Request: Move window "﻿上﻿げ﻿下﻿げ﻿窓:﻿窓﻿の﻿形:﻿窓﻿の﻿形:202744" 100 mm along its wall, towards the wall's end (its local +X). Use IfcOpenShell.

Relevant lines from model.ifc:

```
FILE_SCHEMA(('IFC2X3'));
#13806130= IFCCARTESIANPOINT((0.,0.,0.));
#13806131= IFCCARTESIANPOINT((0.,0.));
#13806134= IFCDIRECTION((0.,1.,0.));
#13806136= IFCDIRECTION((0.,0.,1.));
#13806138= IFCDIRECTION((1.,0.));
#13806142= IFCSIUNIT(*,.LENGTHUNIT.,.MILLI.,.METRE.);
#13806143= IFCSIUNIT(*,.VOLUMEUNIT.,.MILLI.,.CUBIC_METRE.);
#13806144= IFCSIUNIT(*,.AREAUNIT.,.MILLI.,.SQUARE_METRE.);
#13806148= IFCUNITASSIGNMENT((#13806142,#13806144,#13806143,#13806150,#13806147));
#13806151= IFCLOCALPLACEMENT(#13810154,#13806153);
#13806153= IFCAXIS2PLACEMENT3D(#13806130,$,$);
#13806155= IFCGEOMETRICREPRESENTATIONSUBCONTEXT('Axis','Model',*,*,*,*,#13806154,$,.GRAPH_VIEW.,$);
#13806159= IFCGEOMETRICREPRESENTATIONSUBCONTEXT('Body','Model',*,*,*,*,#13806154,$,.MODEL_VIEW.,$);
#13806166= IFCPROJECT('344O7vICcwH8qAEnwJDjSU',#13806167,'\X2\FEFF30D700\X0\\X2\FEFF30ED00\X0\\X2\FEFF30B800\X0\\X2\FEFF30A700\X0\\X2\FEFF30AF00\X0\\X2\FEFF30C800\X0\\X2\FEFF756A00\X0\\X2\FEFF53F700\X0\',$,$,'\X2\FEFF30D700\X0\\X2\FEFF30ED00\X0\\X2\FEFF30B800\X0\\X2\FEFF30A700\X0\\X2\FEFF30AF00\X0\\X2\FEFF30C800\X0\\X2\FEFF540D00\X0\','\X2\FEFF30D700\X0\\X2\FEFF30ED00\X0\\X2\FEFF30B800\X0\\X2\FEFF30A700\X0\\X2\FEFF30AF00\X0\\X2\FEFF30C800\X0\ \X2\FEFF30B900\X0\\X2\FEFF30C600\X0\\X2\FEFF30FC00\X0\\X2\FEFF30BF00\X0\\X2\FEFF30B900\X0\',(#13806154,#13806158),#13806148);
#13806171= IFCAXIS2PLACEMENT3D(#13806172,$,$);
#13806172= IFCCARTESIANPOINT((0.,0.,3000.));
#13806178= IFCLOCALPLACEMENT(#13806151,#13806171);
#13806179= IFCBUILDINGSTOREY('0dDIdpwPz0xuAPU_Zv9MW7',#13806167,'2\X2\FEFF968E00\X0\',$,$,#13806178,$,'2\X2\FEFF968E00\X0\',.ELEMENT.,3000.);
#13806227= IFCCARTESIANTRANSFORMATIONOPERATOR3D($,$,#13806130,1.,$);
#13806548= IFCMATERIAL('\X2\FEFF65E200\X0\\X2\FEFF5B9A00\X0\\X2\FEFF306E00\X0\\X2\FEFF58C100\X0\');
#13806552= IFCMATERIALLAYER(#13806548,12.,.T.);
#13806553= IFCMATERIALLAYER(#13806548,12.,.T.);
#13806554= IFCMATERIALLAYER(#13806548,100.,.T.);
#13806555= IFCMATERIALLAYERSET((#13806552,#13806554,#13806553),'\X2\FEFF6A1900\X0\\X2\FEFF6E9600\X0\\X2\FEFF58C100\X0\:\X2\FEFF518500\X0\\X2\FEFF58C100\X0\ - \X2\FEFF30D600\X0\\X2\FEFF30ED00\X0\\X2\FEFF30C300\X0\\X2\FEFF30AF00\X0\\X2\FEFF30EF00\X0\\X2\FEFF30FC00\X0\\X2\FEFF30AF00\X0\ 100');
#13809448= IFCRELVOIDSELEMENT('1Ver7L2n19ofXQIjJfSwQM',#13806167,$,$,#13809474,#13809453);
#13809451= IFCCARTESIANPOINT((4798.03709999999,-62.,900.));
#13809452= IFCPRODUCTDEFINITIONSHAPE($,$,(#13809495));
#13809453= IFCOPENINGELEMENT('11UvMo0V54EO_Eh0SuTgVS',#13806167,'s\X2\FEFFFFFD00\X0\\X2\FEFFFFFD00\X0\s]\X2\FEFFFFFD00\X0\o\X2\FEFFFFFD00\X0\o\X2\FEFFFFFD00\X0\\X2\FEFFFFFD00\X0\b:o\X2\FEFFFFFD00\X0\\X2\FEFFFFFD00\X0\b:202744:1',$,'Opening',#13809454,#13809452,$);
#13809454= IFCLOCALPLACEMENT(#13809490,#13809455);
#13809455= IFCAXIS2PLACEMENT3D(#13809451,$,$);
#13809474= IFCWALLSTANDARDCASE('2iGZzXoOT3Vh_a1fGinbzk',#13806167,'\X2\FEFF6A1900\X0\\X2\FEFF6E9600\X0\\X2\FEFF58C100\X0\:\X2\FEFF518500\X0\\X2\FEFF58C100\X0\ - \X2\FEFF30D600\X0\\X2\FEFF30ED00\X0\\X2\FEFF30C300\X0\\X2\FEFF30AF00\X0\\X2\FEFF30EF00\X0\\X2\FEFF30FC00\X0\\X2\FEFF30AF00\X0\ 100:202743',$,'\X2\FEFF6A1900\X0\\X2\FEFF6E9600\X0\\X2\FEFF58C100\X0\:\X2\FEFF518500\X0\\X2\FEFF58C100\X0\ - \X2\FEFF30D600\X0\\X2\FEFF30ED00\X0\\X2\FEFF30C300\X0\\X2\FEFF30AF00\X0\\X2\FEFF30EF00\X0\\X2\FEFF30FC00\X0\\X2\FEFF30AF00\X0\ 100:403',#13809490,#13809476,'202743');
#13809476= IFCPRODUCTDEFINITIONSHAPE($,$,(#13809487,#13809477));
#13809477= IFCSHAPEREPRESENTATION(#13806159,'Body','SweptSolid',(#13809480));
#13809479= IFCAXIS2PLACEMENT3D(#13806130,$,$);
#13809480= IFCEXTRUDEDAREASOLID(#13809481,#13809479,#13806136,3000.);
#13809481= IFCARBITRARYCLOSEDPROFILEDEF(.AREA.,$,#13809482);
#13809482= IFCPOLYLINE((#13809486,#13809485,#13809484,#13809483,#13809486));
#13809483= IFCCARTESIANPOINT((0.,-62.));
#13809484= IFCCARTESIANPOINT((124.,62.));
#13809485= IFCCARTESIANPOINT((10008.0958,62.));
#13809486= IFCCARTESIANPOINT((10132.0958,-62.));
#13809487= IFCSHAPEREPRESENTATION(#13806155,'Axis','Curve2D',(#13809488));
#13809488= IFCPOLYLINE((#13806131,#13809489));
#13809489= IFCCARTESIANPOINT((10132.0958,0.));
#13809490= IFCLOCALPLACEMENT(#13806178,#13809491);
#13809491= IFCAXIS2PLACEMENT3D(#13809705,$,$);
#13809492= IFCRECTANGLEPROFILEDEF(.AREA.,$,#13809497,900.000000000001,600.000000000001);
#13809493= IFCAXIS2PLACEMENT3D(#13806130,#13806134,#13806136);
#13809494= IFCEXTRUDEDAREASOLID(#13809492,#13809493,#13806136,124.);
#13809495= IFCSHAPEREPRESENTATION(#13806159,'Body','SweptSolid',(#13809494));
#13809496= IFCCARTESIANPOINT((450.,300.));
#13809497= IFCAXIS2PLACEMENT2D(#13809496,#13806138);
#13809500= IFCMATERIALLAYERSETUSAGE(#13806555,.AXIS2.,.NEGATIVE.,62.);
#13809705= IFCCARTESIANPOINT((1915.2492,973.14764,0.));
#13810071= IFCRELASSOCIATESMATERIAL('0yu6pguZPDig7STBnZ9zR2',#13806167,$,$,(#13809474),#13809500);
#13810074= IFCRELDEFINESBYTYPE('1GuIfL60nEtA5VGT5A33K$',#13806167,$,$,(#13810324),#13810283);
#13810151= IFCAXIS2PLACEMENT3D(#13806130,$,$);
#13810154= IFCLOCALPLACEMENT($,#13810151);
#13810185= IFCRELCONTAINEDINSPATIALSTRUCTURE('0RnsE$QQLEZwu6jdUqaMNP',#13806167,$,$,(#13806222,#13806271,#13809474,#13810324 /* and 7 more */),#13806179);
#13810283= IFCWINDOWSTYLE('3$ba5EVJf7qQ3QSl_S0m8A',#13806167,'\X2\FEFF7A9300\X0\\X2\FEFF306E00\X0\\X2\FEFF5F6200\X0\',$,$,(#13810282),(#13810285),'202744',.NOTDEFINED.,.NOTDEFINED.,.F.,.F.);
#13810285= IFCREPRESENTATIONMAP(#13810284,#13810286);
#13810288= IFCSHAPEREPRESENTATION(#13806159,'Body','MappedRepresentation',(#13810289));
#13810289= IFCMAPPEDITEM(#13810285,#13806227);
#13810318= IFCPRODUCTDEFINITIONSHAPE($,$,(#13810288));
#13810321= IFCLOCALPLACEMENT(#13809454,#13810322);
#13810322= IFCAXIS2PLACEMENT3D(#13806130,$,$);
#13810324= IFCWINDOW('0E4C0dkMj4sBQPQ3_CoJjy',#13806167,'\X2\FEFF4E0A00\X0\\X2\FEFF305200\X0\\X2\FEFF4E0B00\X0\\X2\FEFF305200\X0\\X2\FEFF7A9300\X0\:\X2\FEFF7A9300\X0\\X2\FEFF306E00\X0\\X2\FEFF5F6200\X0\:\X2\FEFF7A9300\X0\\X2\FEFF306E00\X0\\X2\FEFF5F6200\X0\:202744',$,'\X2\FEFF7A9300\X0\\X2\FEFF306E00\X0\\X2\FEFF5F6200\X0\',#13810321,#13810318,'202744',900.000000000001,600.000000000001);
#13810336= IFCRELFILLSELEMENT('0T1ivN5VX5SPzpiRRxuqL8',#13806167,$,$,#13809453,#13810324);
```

```python
import ifcopenshell
import ifcopenshell.api.geometry
import ifcopenshell.util.placement
import ifcopenshell.util.unit

model = ifcopenshell.open("model.ifc")
unit_scale = ifcopenshell.util.unit.calculate_unit_scale(model)

window = model.by_guid("0E4C0dkMj4sBQPQ3_CoJjy")
opening = window.FillsVoids[0].RelatingOpeningElement
wall = opening.VoidsElements[0].RelatingBuildingElement

wall_matrix = ifcopenshell.util.placement.get_local_placement(wall.ObjectPlacement)
shift = wall_matrix[:3, 0] * 0.1 / unit_scale
before = ifcopenshell.util.placement.get_local_placement(window.ObjectPlacement)[:3, 3].copy()

# The window is placed relative to its opening, so it follows when the opening moves.
matrix = ifcopenshell.util.placement.get_local_placement(opening.ObjectPlacement)
matrix[:3, 3] += shift
ifcopenshell.api.geometry.edit_object_placement(
    model, product=opening, matrix=matrix, is_si=False, should_transform_children=True
)

after = ifcopenshell.util.placement.get_local_placement(window.ObjectPlacement)[:3, 3]
print("window moved by", (after - before).round(3) + 0.0)

model.write("model_edited.ifc")
```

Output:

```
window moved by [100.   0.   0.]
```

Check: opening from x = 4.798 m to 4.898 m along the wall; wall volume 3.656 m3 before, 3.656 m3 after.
